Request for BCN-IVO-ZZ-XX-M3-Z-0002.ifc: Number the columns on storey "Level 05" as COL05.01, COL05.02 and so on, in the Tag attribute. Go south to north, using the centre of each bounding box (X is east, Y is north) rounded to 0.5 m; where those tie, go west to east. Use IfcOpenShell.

First a look at what the model holds.

```python
import ifcopenshell
import ifcopenshell.util.element
import ifcopenshell.util.placement

model = ifcopenshell.open("BCN-IVO-ZZ-XX-M3-Z-0002.ifc")
print(model.schema)
storey = next(s for s in model.by_type("IfcBuildingStorey") if s.Name == "Level 05")
columns = [e for e in ifcopenshell.util.element.get_decomposition(storey) if e.is_a("IfcColumn")]
for e in sorted(columns, key=lambda e: e.id()):
    origin = ifcopenshell.util.placement.get_local_placement(e.ObjectPlacement)[:3, 3]
    print(e.id(), e.Tag, e.Name, origin.round(2) + 0.0, sep=" | ")
```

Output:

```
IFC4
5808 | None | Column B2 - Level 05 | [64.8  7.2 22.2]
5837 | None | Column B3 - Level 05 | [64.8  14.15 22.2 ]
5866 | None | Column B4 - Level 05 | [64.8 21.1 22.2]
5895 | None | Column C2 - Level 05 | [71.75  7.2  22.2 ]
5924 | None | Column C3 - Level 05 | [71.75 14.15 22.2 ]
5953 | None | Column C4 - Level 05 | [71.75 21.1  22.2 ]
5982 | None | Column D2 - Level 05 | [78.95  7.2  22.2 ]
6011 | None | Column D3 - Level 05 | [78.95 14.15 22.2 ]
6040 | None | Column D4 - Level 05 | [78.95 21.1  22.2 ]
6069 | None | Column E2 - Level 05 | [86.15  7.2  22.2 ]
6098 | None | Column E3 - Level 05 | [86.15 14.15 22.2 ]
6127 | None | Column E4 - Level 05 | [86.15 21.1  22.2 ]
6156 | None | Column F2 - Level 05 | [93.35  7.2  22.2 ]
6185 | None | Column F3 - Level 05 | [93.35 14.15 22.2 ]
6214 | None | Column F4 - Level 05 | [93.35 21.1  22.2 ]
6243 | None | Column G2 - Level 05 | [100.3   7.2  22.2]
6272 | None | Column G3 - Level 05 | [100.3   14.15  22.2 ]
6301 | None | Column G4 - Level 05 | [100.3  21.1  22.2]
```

```python
import ifcopenshell
import ifcopenshell.geom
import ifcopenshell.util.element
import ifcopenshell.util.shape

model = ifcopenshell.open("BCN-IVO-ZZ-XX-M3-Z-0002.ifc")
settings = ifcopenshell.geom.settings()
settings.set("use-world-coords", True)


def centre(element):
    shape = ifcopenshell.geom.create_shape(settings, element)
    return ifcopenshell.util.shape.get_bbox_centroid(shape.geometry)


storey = next(s for s in model.by_type("IfcBuildingStorey") if s.Name == "Level 05")
columns = [e for e in ifcopenshell.util.element.get_decomposition(storey) if e.is_a("IfcColumn")]

# Insertion points can sit at a corner or the storey origin, so sort by the geometry (in metres).
centres = {e: centre(e) for e in columns}
columns.sort(key=lambda e: (round(centres[e][1] / 0.5), centres[e][0]))

for i, e in enumerate(columns, start=1):
    number = f"COL05.{i:02d}"
    e.Tag = number
    print(e.id(), number)

model.write("BCN-IVO-ZZ-XX-M3-Z-0002_updated.ifc")
```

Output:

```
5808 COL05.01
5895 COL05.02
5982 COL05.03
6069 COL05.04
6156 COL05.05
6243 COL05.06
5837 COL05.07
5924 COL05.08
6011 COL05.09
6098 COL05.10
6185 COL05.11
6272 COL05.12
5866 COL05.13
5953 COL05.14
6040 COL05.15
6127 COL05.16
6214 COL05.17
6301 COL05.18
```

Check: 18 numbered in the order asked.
